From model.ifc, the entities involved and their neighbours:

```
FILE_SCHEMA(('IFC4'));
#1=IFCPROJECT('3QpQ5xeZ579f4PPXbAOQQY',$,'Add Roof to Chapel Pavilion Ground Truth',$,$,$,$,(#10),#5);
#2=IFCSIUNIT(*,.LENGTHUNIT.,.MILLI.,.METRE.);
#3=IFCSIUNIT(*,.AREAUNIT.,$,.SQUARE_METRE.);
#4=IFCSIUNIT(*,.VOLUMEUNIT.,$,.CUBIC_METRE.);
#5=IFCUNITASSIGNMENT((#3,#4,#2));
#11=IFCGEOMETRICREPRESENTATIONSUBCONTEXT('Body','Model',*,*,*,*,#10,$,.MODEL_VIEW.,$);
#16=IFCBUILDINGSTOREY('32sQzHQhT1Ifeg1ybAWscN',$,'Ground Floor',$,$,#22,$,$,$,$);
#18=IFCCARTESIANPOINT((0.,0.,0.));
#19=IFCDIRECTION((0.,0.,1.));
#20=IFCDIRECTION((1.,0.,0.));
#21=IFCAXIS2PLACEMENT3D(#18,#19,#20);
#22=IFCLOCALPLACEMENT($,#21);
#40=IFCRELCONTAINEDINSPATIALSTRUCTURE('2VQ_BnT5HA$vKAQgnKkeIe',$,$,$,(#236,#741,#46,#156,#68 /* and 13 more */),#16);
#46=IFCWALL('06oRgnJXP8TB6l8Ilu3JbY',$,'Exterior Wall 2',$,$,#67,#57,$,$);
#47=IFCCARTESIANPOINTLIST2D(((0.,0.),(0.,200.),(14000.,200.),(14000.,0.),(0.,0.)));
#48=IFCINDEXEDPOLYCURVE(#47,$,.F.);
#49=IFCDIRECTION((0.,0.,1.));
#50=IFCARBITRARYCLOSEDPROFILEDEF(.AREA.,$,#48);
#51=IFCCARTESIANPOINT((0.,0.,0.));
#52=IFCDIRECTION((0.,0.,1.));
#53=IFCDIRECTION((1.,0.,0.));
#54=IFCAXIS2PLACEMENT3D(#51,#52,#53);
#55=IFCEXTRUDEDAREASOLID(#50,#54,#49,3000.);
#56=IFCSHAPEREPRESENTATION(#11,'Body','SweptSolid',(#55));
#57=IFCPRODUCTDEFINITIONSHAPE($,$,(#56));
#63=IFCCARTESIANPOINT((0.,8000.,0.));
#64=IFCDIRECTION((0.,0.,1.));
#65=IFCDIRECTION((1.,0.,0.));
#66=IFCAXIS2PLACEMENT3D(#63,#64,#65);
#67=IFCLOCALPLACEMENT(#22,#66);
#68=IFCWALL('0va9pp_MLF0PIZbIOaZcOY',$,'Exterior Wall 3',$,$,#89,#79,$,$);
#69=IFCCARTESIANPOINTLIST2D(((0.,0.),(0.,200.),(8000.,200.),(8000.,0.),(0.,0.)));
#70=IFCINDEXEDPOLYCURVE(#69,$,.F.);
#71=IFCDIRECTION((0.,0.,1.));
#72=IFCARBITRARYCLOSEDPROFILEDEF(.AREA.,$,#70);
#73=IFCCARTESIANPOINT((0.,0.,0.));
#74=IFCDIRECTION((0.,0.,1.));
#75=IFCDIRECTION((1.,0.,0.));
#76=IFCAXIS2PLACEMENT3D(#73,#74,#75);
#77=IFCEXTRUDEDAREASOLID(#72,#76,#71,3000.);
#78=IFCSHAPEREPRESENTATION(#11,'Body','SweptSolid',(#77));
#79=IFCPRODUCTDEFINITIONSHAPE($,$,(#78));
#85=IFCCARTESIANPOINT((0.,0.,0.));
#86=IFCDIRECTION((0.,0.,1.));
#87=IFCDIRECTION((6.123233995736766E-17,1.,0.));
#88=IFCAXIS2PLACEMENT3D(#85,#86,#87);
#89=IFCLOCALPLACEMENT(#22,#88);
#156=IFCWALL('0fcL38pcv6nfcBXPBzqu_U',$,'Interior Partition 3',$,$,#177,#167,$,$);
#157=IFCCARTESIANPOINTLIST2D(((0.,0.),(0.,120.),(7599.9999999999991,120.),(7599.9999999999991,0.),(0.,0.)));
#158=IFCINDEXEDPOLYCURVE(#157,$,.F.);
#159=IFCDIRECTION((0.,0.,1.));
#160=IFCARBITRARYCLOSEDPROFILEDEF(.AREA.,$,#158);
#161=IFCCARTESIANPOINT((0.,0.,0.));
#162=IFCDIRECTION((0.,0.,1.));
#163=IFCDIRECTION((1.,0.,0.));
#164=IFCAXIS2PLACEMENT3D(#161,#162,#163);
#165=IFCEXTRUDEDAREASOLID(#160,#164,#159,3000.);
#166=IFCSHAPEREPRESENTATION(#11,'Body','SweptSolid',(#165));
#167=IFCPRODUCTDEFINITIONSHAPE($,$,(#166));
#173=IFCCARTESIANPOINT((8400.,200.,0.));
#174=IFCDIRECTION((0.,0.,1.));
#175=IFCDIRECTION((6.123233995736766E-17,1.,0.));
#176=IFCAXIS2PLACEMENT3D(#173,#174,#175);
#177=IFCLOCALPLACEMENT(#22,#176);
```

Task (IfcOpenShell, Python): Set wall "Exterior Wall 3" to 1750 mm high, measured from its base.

```python
import ifcopenshell
import ifcopenshell.geom
import ifcopenshell.util.representation
import ifcopenshell.util.shape

model = ifcopenshell.open("model.ifc")
settings = ifcopenshell.geom.settings()


def volume(element):
    """Net volume in cubic metres, openings subtracted."""
    shape = ifcopenshell.geom.create_shape(settings, element)
    return ifcopenshell.util.shape.get_volume(shape.geometry)


wall = model.by_guid("0va9pp_MLF0PIZbIOaZcOY")
before = volume(wall)

body = ifcopenshell.util.representation.get_representation(wall, "Model", "Body")
solid = body.Items[0]
old_height = solid.Depth
solid.Depth = 1750.0
after = volume(wall)

print(f"height {old_height:g} -> {solid.Depth:g}, volume {before:.3f} -> {after:.3f} m3")

model.write("model-out.ifc")
```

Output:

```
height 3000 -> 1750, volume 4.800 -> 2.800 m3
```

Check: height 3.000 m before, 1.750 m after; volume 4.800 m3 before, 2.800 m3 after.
